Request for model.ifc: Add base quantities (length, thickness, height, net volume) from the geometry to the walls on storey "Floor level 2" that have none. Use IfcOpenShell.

First a look at what the model holds.

```python
import ifcopenshell
import ifcopenshell.util.element
import ifcopenshell.util.unit

model = ifcopenshell.open("model.ifc")
print(model.schema)
for unit_type in ("LENGTHUNIT", "AREAUNIT", "VOLUMEUNIT"):
    print(unit_type, ifcopenshell.util.unit.calculate_unit_scale(model, unit_type))
storey = next(s for s in model.by_type("IfcBuildingStorey") if s.Name == "Floor level 2")
walls = [e for e in ifcopenshell.util.element.get_decomposition(storey) if e.is_a("IfcWall")]
for e in sorted(walls, key=lambda e: e.id()):
    print(e.id(), e.is_a(), e.Name, list(ifcopenshell.util.element.get_psets(e, qtos_only=True)), sep=" | ")
```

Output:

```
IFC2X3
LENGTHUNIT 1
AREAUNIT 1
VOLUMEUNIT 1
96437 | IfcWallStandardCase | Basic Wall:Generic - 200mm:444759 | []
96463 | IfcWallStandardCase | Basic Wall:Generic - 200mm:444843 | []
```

```python
import ifcopenshell
import ifcopenshell.api.pset
import ifcopenshell.geom
import ifcopenshell.util.element
import ifcopenshell.util.shape
import ifcopenshell.util.unit

model = ifcopenshell.open("model.ifc")
unit_scale = ifcopenshell.util.unit.calculate_unit_scale(model)
volume_scale = ifcopenshell.util.unit.calculate_unit_scale(model, "VOLUMEUNIT")
settings = ifcopenshell.geom.settings()

storey = next(s for s in model.by_type("IfcBuildingStorey") if s.Name == "Floor level 2")
walls = [e for e in ifcopenshell.util.element.get_decomposition(storey) if e.is_a("IfcWall")]

for e in sorted(walls, key=lambda e: e.id()):
    if ifcopenshell.util.element.get_psets(e, qtos_only=True, should_inherit=False):
        continue
    # Geometry comes back in metres, in the element's own axes.
    shape = ifcopenshell.geom.create_shape(settings, e)
    values = {
        "Length": ifcopenshell.util.shape.get_x(shape.geometry) / unit_scale,
        "Width": ifcopenshell.util.shape.get_y(shape.geometry) / unit_scale,
        "Height": ifcopenshell.util.shape.get_z(shape.geometry) / unit_scale,
        "NetVolume": ifcopenshell.util.shape.get_volume(shape.geometry) / volume_scale,
    }
    qto = ifcopenshell.api.pset.add_qto(model, product=e, name="BaseQuantities")
    ifcopenshell.api.pset.edit_qto(model, qto=qto, properties=values)
    print(e.id(), {k: round(v, 3) for k, v in values.items()})

model.write("model_v2.ifc")
```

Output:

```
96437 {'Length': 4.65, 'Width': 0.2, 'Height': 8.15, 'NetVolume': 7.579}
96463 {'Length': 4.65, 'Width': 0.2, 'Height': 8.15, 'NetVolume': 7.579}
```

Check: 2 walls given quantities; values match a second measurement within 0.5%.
